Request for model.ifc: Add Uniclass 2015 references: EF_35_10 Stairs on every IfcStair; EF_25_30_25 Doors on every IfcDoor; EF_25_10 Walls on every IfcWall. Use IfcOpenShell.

First a look at what the model holds.

```python
import ifcopenshell

model = ifcopenshell.open("model.ifc")
print(model.schema)
print("classifications:", [c.Name for c in model.by_type("IfcClassification")])
for ifc_class in ("IfcDoor", "IfcRoof", "IfcStair", "IfcWall", "IfcWindow"):
    print(ifc_class, len(model.by_type(ifc_class)))
```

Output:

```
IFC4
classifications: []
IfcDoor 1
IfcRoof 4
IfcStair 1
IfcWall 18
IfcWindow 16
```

```python
import ifcopenshell
import ifcopenshell.api.classification

model = ifcopenshell.open("model.ifc")

system = ifcopenshell.api.classification.add_classification(model, classification="Uniclass 2015")

codes = {
    "IfcStair": ("EF_35_10", "Stairs"),
    "IfcDoor": ("EF_25_30_25", "Doors"),
    "IfcWall": ("EF_25_10", "Walls"),
}
for ifc_class, (code, name) in codes.items():
    products = model.by_type(ifc_class)
    ifcopenshell.api.classification.add_reference(
        model, products=products, classification=system, identification=code, name=name
    )
    print(code, len(products))

model.write("model_updated.ifc")
```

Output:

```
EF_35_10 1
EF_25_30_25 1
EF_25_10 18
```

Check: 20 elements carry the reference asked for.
